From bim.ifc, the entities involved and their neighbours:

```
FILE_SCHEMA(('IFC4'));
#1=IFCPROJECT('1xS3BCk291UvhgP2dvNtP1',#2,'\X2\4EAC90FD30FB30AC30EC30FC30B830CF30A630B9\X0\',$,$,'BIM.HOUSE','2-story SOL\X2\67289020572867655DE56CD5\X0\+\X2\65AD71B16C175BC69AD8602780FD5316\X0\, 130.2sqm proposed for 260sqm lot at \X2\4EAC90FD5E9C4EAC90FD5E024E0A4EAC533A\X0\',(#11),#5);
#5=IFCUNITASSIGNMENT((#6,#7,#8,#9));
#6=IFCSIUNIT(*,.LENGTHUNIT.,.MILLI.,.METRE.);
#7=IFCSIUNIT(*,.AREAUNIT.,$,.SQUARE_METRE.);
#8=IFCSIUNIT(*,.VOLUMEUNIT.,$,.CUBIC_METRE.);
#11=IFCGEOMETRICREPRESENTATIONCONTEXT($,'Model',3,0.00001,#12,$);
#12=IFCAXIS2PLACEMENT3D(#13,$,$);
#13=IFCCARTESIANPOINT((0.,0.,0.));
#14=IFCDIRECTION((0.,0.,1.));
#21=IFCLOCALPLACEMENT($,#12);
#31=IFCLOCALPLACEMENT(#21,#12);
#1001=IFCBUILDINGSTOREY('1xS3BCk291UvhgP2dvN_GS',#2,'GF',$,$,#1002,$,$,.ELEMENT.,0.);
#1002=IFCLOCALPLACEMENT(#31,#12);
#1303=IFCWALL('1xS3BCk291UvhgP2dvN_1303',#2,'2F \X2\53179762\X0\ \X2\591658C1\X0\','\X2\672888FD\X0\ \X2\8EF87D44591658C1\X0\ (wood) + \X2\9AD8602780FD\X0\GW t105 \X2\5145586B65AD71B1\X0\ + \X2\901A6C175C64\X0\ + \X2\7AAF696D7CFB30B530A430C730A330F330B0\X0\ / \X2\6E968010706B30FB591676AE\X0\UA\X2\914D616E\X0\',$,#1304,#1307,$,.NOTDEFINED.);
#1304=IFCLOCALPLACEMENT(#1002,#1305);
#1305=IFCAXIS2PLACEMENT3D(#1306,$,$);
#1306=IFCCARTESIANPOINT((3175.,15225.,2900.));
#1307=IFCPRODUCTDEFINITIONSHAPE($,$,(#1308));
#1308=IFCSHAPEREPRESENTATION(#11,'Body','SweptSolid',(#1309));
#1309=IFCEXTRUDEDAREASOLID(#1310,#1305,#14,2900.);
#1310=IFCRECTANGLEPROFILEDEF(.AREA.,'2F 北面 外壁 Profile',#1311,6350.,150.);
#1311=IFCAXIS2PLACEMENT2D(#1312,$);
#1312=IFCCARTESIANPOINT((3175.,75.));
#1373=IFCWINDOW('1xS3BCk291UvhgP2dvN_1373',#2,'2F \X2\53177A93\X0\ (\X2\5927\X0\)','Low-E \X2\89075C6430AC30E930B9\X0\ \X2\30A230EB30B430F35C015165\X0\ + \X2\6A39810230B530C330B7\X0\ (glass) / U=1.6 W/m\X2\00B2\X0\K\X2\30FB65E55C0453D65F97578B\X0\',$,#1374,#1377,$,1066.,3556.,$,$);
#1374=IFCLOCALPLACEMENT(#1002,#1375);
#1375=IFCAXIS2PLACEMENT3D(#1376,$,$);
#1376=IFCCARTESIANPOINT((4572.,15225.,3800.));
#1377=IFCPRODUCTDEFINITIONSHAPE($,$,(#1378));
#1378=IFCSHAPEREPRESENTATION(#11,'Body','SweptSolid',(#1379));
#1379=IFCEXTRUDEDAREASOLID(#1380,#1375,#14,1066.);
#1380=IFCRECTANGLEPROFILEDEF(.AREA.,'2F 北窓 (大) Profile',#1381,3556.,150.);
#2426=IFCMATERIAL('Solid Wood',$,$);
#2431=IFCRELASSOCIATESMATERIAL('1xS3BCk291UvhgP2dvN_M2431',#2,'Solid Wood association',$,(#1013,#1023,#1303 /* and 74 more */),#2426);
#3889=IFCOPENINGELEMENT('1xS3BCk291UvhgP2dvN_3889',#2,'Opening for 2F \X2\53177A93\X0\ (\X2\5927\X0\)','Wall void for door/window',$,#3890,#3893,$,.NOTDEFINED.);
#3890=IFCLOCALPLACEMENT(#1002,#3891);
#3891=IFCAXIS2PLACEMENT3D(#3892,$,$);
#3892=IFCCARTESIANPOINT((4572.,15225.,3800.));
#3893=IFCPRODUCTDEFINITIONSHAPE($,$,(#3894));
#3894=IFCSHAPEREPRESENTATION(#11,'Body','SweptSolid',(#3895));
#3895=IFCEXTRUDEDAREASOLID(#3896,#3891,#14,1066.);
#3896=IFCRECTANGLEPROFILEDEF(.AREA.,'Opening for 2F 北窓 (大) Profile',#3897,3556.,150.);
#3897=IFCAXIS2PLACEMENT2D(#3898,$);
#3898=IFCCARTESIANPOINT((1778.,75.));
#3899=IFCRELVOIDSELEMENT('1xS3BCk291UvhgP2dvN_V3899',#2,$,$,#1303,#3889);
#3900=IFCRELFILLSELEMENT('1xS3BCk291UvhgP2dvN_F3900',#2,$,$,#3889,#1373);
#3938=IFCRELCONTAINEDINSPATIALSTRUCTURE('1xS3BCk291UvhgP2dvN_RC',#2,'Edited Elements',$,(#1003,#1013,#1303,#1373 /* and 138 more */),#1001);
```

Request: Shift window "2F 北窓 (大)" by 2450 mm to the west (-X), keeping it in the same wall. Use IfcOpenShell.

```python
import ifcopenshell
import ifcopenshell.api.geometry
import ifcopenshell.util.placement

model = ifcopenshell.open("bim.ifc")

window = model.by_id(1373)
opening = window.FillsVoids[0].RelatingOpeningElement
wall = opening.VoidsElements[0].RelatingBuildingElement

wall_matrix = ifcopenshell.util.placement.get_local_placement(wall.ObjectPlacement)
shift = wall_matrix[:3, 0] * -2450.0
before = ifcopenshell.util.placement.get_local_placement(window.ObjectPlacement)[:3, 3].copy()

# The window is not placed relative to its opening, so move both.
for product in (opening, window):
    matrix = ifcopenshell.util.placement.get_local_placement(product.ObjectPlacement)
    matrix[:3, 3] += shift
    ifcopenshell.api.geometry.edit_object_placement(model, product=product, matrix=matrix, is_si=False)

after = ifcopenshell.util.placement.get_local_placement(window.ObjectPlacement)[:3, 3]
print("window moved by", (after - before).round(3) + 0.0)

model.write("bim_rev.ifc")
```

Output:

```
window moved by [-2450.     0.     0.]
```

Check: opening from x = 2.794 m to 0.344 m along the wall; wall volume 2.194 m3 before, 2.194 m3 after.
